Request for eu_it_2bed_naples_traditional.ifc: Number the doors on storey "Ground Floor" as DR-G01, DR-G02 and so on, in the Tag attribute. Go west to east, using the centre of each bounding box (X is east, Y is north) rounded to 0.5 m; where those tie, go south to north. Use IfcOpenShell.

First a look at what the model holds.

```python
import ifcopenshell
import ifcopenshell.util.element
import ifcopenshell.util.placement

model = ifcopenshell.open("eu_it_2bed_naples_traditional.ifc")
print(model.schema)
storey = next(s for s in model.by_type("IfcBuildingStorey") if s.Name == "Ground Floor")
doors = [e for e in ifcopenshell.util.element.get_decomposition(storey) if e.is_a("IfcDoor")]
for e in sorted(doors, key=lambda e: e.id()):
    origin = ifcopenshell.util.placement.get_local_placement(e.ObjectPlacement)[:3, 3]
    print(e.id(), e.Tag, e.Name, origin.round(2) + 0.0, sep=" | ")
```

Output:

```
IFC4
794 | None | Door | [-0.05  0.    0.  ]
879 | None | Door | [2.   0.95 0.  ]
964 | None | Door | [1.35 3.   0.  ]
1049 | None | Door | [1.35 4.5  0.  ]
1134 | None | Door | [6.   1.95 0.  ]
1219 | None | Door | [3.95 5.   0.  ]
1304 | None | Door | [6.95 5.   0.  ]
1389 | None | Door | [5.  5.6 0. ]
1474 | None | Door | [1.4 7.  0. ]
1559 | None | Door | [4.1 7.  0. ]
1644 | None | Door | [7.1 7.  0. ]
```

```python
import ifcopenshell
import ifcopenshell.geom
import ifcopenshell.util.element
import ifcopenshell.util.shape

model = ifcopenshell.open("eu_it_2bed_naples_traditional.ifc")
settings = ifcopenshell.geom.settings()
settings.set("use-world-coords", True)


def centre(element):
    shape = ifcopenshell.geom.create_shape(settings, element)
    return ifcopenshell.util.shape.get_bbox_centroid(shape.geometry)


storey = next(s for s in model.by_type("IfcBuildingStorey") if s.Name == "Ground Floor")
doors = [e for e in ifcopenshell.util.element.get_decomposition(storey) if e.is_a("IfcDoor")]

# Insertion points can sit at a corner or the storey origin, so sort by the geometry (in metres).
centres = {e: centre(e) for e in doors}
doors.sort(key=lambda e: (round(centres[e][0] / 0.5), centres[e][1]))

for i, e in enumerate(doors, start=1):
    number = f"DR-G{i:02d}"
    e.Tag = number
    print(e.id(), number)

model.write("eu_it_2bed_naples_traditional_edited.ifc")
```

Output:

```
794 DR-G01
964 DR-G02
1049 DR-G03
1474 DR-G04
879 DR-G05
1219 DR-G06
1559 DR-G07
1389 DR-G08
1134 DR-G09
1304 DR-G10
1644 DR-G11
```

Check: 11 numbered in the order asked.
